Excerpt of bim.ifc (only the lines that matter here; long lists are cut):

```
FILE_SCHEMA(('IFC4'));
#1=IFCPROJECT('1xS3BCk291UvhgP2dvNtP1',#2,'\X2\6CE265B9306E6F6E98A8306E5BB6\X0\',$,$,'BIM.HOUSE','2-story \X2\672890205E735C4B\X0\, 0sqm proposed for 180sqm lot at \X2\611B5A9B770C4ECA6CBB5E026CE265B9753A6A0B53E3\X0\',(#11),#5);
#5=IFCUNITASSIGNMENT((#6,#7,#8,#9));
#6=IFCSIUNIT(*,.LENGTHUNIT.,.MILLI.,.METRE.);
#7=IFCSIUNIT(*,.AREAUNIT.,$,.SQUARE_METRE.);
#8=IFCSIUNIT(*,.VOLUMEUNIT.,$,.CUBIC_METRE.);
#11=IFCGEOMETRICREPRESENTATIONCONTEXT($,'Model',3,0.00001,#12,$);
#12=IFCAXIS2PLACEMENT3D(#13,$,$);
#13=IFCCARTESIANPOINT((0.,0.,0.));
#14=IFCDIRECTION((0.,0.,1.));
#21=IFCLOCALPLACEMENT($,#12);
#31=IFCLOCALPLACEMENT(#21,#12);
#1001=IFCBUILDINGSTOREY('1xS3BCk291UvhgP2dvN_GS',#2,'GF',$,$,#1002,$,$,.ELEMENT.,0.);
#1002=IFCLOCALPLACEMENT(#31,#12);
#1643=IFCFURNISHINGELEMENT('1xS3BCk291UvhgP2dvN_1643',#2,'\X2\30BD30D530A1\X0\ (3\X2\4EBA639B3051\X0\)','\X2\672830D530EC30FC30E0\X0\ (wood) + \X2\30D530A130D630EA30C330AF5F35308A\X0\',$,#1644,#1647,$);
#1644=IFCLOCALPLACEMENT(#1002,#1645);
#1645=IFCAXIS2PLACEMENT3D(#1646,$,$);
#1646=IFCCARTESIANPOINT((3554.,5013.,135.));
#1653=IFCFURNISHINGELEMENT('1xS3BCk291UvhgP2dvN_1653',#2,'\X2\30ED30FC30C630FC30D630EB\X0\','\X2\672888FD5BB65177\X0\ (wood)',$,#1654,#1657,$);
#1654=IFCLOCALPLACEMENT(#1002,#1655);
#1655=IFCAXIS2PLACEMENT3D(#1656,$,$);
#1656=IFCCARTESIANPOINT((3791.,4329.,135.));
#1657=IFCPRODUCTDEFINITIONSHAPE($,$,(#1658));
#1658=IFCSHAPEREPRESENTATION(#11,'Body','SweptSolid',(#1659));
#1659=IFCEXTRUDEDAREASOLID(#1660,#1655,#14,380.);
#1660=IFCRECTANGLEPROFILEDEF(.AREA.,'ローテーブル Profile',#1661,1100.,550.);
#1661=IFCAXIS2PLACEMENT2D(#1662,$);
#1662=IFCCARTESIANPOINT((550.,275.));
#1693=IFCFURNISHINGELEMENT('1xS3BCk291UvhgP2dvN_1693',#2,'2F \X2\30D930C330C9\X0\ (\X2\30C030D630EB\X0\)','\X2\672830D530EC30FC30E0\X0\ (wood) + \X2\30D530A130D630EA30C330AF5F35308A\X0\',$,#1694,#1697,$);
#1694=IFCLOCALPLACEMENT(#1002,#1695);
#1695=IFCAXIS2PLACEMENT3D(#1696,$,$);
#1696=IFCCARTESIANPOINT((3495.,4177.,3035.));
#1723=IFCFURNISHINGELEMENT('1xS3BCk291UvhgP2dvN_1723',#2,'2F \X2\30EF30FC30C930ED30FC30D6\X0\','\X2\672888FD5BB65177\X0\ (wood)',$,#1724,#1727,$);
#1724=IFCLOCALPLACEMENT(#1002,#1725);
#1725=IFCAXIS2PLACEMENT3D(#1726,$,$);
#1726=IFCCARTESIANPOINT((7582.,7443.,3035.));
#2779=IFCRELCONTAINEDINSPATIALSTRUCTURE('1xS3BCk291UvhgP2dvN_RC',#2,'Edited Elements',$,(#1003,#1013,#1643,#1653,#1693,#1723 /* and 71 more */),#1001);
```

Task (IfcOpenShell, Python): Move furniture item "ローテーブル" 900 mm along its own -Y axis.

```python
import ifcopenshell
import ifcopenshell.api.geometry
import ifcopenshell.util.placement

model = ifcopenshell.open("bim.ifc")

item = model.by_guid("1xS3BCk291UvhgP2dvN_1653")
matrix = ifcopenshell.util.placement.get_local_placement(item.ObjectPlacement)
matrix[:3, 3] -= matrix[:3, 1] * 900.0
ifcopenshell.api.geometry.edit_object_placement(model, product=item, matrix=matrix, is_si=False)

print(ifcopenshell.util.placement.get_local_placement(item.ObjectPlacement).round(3) + 0.0)

model.write("bim_edited.ifc")
```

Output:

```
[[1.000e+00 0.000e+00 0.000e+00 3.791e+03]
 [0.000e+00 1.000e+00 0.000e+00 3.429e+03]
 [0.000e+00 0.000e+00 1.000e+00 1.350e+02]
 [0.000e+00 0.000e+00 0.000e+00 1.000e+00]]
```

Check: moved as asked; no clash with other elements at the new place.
